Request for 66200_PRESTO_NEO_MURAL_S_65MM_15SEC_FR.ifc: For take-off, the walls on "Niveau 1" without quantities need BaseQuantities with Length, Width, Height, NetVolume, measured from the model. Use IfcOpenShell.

First a look at what the model holds.

```python
import ifcopenshell
import ifcopenshell.util.element
import ifcopenshell.util.unit

model = ifcopenshell.open("66200_PRESTO_NEO_MURAL_S_65MM_15SEC_FR.ifc")
print(model.schema)
for unit_type in ("LENGTHUNIT", "AREAUNIT", "VOLUMEUNIT"):
    print(unit_type, ifcopenshell.util.unit.calculate_unit_scale(model, unit_type))
storey = next(s for s in model.by_type("IfcBuildingStorey") if s.Name == "Niveau 1")
walls = [e for e in ifcopenshell.util.element.get_decomposition(storey) if e.is_a("IfcWall")]
for e in sorted(walls, key=lambda e: e.id()):
    print(e.id(), e.is_a(), e.Name, list(ifcopenshell.util.element.get_psets(e, qtos_only=True)), sep=" | ")
```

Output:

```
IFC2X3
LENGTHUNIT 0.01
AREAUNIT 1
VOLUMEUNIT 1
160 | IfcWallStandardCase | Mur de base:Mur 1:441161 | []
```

```python
import ifcopenshell
import ifcopenshell.api.pset
import ifcopenshell.geom
import ifcopenshell.util.element
import ifcopenshell.util.shape
import ifcopenshell.util.unit

model = ifcopenshell.open("66200_PRESTO_NEO_MURAL_S_65MM_15SEC_FR.ifc")
unit_scale = ifcopenshell.util.unit.calculate_unit_scale(model)
volume_scale = ifcopenshell.util.unit.calculate_unit_scale(model, "VOLUMEUNIT")
settings = ifcopenshell.geom.settings()

storey = next(s for s in model.by_type("IfcBuildingStorey") if s.Name == "Niveau 1")
walls = [e for e in ifcopenshell.util.element.get_decomposition(storey) if e.is_a("IfcWall")]

for e in sorted(walls, key=lambda e: e.id()):
    if ifcopenshell.util.element.get_psets(e, qtos_only=True, should_inherit=False):
        continue
    # Geometry comes back in metres, in the element's own axes.
    shape = ifcopenshell.geom.create_shape(settings, e)
    values = {
        "Length": ifcopenshell.util.shape.get_x(shape.geometry) / unit_scale,
        "Width": ifcopenshell.util.shape.get_y(shape.geometry) / unit_scale,
        "Height": ifcopenshell.util.shape.get_z(shape.geometry) / unit_scale,
        "NetVolume": ifcopenshell.util.shape.get_volume(shape.geometry) / volume_scale,
    }
    qto = ifcopenshell.api.pset.add_qto(model, product=e, name="BaseQuantities")
    ifcopenshell.api.pset.edit_qto(model, qto=qto, properties=values)
    print(e.id(), {k: round(v, 3) for k, v in values.items()})

model.write("66200_PRESTO_NEO_MURAL_S_65MM_15SEC_FR_edited.ifc")
```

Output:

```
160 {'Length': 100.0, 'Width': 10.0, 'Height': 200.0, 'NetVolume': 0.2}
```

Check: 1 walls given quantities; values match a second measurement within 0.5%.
